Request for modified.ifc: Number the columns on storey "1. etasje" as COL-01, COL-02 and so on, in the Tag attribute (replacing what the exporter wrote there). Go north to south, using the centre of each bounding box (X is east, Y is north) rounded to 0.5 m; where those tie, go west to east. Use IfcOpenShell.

First a look at what the model holds.

```python
import ifcopenshell
import ifcopenshell.util.element
import ifcopenshell.util.placement

model = ifcopenshell.open("modified.ifc")
print(model.schema)
storey = next(s for s in model.by_type("IfcBuildingStorey") if s.Name == "1. etasje")
columns = [e for e in ifcopenshell.util.element.get_decomposition(storey) if e.is_a("IfcColumn")]
for e in sorted(columns, key=lambda e: e.id()):
    origin = ifcopenshell.util.placement.get_local_placement(e.ObjectPlacement)[:3, 3]
    print(e.id(), e.Tag, e.Name, origin.round(2) + 0.0, sep=" | ")
```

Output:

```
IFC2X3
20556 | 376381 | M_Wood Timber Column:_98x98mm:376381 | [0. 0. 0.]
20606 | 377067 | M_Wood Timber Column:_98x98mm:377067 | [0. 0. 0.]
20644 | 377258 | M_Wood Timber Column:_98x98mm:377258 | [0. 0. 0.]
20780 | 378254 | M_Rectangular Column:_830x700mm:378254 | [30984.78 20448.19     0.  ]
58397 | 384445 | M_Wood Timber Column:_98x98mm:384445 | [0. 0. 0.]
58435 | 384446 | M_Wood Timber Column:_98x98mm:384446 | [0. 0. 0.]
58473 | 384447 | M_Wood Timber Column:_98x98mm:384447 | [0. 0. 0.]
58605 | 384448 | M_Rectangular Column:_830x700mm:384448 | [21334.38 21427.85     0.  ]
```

```python
import ifcopenshell
import ifcopenshell.geom
import ifcopenshell.util.element
import ifcopenshell.util.shape

model = ifcopenshell.open("modified.ifc")
settings = ifcopenshell.geom.settings()
settings.set("use-world-coords", True)


def centre(element):
    shape = ifcopenshell.geom.create_shape(settings, element)
    return ifcopenshell.util.shape.get_bbox_centroid(shape.geometry)


storey = next(s for s in model.by_type("IfcBuildingStorey") if s.Name == "1. etasje")
columns = [e for e in ifcopenshell.util.element.get_decomposition(storey) if e.is_a("IfcColumn")]

# Insertion points can sit at a corner or the storey origin, so sort by the geometry (in metres).
centres = {e: centre(e) for e in columns}
columns.sort(key=lambda e: (-round(centres[e][1] / 0.5), centres[e][0]))

for i, e in enumerate(columns, start=1):
    number = f"COL-{i:02d}"
    e.Tag = number
    print(e.id(), number)

model.write("modified_updated.ifc")
```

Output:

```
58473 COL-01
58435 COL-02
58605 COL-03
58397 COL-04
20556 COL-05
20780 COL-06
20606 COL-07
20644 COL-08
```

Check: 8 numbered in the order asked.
